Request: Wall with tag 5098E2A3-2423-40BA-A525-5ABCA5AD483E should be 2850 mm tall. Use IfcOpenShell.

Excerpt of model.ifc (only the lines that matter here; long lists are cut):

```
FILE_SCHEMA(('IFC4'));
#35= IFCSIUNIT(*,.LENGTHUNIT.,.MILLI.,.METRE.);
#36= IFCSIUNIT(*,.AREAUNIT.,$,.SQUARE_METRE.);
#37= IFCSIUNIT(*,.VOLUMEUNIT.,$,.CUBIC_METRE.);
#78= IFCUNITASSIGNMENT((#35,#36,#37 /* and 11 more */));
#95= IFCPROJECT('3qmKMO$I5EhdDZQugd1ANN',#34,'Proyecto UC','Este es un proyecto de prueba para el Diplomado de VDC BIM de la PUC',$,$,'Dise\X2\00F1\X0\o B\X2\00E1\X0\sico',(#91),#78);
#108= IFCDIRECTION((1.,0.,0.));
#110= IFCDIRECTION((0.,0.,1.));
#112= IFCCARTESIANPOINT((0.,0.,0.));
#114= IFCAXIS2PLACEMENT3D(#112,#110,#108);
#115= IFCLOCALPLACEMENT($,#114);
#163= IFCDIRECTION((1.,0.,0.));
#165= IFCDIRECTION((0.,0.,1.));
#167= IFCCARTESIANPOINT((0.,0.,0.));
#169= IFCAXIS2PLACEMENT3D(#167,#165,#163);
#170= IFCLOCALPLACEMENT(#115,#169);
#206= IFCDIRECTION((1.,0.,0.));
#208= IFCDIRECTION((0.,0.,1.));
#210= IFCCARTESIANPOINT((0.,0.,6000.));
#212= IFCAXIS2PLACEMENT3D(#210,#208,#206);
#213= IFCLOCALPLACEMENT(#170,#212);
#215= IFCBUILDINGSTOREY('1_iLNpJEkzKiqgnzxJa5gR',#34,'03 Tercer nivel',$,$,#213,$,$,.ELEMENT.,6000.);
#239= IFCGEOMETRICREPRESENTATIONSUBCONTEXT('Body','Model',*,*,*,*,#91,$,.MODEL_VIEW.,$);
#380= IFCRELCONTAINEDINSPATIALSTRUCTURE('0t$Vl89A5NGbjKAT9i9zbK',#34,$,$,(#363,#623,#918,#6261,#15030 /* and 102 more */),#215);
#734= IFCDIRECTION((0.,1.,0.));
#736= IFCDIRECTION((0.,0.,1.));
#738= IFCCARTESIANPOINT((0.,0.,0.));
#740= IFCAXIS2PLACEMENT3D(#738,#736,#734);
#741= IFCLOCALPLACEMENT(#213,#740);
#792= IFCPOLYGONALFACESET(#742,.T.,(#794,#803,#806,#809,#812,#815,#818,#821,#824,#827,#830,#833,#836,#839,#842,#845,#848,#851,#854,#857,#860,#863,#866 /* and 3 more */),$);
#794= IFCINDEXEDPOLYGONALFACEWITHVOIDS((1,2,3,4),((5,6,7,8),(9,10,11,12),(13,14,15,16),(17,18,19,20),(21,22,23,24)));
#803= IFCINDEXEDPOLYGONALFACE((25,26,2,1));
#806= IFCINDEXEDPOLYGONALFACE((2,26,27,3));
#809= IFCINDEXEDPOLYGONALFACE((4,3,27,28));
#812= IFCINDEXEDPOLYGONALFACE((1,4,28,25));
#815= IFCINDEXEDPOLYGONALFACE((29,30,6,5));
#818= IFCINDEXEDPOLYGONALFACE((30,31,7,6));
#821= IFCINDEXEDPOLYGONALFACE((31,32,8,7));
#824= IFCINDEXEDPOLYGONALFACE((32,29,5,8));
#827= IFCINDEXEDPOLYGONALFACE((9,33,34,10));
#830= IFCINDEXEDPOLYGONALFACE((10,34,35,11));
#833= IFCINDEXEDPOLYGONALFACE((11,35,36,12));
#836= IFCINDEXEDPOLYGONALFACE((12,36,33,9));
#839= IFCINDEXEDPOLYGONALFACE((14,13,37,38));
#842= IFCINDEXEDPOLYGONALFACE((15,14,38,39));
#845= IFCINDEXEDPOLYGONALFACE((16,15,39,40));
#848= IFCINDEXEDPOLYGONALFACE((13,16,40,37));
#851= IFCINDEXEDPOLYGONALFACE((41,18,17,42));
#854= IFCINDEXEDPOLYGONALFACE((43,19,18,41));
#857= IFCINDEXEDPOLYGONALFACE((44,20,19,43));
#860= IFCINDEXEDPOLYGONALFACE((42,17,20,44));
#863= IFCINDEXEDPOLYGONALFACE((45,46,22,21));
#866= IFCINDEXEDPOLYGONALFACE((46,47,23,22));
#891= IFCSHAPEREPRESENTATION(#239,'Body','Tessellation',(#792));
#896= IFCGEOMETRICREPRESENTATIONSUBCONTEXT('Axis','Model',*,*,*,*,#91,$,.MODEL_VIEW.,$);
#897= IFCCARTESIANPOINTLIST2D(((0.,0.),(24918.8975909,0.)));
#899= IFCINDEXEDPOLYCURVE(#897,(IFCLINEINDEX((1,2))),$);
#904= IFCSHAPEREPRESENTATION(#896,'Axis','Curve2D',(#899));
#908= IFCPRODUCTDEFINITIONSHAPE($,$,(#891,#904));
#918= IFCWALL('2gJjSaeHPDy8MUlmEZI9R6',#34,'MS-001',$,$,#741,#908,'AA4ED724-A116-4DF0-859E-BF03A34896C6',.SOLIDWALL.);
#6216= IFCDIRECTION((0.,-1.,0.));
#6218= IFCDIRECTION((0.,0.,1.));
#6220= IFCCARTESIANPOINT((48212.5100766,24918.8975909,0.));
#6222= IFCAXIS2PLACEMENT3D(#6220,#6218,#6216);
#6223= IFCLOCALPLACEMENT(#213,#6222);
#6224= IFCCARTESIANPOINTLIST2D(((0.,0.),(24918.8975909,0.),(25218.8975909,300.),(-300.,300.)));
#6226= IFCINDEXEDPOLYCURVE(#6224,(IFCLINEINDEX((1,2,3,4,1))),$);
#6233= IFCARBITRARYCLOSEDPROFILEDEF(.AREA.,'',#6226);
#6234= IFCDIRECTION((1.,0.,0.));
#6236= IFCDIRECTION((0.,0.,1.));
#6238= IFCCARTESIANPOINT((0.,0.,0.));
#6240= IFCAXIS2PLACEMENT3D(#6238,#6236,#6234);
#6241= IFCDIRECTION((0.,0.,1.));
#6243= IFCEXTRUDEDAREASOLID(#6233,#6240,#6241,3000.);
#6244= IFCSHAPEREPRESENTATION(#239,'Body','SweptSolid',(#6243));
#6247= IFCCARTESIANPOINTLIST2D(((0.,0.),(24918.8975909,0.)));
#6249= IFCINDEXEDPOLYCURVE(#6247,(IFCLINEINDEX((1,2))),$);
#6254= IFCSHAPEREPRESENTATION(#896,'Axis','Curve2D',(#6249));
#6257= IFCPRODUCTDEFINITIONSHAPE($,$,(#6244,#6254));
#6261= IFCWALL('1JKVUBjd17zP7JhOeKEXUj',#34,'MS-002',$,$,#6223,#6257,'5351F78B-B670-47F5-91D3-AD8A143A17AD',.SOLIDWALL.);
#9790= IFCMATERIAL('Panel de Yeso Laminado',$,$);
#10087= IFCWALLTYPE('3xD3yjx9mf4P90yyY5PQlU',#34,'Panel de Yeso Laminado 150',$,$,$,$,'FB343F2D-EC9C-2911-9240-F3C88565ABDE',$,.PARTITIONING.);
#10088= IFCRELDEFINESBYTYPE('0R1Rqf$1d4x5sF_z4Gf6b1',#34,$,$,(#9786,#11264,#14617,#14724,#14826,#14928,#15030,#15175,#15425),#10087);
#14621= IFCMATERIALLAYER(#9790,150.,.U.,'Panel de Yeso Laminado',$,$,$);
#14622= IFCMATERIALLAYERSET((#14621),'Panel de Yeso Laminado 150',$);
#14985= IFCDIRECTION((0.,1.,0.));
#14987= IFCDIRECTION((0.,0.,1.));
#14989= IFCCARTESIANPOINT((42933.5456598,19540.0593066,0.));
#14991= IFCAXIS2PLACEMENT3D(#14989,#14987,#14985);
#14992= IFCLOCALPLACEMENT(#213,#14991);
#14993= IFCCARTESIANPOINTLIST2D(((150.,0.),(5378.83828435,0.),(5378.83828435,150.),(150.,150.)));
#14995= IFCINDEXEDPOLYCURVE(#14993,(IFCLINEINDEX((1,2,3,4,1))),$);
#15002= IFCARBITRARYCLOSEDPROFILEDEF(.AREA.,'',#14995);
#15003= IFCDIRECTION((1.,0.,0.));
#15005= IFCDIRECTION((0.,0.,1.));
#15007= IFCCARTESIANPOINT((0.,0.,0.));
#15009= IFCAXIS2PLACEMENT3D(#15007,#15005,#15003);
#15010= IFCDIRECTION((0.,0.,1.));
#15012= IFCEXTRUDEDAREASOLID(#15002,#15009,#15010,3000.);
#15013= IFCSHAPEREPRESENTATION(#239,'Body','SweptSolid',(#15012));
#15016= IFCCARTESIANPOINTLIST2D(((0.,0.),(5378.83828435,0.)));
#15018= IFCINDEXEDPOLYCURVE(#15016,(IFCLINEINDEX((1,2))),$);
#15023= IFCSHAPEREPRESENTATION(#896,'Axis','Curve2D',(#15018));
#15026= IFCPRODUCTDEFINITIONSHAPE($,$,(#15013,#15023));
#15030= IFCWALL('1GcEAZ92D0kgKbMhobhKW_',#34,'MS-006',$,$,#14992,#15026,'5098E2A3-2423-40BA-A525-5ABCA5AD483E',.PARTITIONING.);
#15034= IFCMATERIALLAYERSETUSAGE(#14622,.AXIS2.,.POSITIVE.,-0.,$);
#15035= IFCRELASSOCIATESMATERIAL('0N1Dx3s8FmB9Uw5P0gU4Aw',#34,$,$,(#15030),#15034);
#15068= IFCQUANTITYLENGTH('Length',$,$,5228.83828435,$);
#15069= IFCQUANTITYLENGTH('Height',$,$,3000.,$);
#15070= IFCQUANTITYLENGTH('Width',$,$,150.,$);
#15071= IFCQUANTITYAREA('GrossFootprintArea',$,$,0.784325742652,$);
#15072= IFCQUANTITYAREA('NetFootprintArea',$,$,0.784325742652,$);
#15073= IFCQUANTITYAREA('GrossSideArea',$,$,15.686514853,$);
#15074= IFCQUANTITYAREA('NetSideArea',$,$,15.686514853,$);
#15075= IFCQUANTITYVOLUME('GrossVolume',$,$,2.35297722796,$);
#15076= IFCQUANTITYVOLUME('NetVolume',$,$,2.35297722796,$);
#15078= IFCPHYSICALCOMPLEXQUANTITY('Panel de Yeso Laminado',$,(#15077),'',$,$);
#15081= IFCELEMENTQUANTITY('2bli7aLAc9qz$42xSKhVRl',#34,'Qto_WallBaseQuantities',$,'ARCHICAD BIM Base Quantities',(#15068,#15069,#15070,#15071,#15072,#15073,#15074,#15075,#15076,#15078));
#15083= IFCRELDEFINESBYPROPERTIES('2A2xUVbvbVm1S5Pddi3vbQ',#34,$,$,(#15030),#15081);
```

```python
import ifcopenshell
import ifcopenshell.api.pset
import ifcopenshell.geom
import ifcopenshell.util.element
import ifcopenshell.util.representation
import ifcopenshell.util.shape
import ifcopenshell.util.unit

model = ifcopenshell.open("model.ifc")
unit_scale = ifcopenshell.util.unit.calculate_unit_scale(model)
area_scale = ifcopenshell.util.unit.calculate_unit_scale(model, "AREAUNIT")
volume_scale = ifcopenshell.util.unit.calculate_unit_scale(model, "VOLUMEUNIT")
settings = ifcopenshell.geom.settings()


def volume(element):
    """Net volume in cubic metres, openings subtracted."""
    shape = ifcopenshell.geom.create_shape(settings, element)
    return ifcopenshell.util.shape.get_volume(shape.geometry)


wall = model.by_guid("1GcEAZ92D0kgKbMhobhKW_")
before = volume(wall)

body = ifcopenshell.util.representation.get_representation(wall, "Model", "Body")
solid = body.Items[0]
old_height = solid.Depth
solid.Depth = 2.85 / unit_scale
after = volume(wall)
thickness = 0.15  # wall thickness in metres

# Update the stored height, areas and volumes.
qto = model.by_id(ifcopenshell.util.element.get_pset(wall, "Qto_WallBaseQuantities", should_inherit=False)["id"])
ifcopenshell.api.pset.edit_qto(model, qto=qto, properties={
    "Height": solid.Depth,
    "GrossSideArea": ifcopenshell.util.element.get_pset(wall, "Qto_WallBaseQuantities", "GrossSideArea") * solid.Depth / old_height,
    "NetSideArea": after / thickness / area_scale,
    "GrossVolume": ifcopenshell.util.element.get_pset(wall, "Qto_WallBaseQuantities", "GrossVolume") * solid.Depth / old_height,
    "NetVolume": after / volume_scale,
})

print(f"height {old_height:g} -> {solid.Depth:g}, volume {before:.3f} -> {after:.3f} m3")

model.write("model_rev.ifc")
```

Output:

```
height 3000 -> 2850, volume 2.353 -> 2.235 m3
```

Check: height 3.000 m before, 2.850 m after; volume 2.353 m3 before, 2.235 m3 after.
